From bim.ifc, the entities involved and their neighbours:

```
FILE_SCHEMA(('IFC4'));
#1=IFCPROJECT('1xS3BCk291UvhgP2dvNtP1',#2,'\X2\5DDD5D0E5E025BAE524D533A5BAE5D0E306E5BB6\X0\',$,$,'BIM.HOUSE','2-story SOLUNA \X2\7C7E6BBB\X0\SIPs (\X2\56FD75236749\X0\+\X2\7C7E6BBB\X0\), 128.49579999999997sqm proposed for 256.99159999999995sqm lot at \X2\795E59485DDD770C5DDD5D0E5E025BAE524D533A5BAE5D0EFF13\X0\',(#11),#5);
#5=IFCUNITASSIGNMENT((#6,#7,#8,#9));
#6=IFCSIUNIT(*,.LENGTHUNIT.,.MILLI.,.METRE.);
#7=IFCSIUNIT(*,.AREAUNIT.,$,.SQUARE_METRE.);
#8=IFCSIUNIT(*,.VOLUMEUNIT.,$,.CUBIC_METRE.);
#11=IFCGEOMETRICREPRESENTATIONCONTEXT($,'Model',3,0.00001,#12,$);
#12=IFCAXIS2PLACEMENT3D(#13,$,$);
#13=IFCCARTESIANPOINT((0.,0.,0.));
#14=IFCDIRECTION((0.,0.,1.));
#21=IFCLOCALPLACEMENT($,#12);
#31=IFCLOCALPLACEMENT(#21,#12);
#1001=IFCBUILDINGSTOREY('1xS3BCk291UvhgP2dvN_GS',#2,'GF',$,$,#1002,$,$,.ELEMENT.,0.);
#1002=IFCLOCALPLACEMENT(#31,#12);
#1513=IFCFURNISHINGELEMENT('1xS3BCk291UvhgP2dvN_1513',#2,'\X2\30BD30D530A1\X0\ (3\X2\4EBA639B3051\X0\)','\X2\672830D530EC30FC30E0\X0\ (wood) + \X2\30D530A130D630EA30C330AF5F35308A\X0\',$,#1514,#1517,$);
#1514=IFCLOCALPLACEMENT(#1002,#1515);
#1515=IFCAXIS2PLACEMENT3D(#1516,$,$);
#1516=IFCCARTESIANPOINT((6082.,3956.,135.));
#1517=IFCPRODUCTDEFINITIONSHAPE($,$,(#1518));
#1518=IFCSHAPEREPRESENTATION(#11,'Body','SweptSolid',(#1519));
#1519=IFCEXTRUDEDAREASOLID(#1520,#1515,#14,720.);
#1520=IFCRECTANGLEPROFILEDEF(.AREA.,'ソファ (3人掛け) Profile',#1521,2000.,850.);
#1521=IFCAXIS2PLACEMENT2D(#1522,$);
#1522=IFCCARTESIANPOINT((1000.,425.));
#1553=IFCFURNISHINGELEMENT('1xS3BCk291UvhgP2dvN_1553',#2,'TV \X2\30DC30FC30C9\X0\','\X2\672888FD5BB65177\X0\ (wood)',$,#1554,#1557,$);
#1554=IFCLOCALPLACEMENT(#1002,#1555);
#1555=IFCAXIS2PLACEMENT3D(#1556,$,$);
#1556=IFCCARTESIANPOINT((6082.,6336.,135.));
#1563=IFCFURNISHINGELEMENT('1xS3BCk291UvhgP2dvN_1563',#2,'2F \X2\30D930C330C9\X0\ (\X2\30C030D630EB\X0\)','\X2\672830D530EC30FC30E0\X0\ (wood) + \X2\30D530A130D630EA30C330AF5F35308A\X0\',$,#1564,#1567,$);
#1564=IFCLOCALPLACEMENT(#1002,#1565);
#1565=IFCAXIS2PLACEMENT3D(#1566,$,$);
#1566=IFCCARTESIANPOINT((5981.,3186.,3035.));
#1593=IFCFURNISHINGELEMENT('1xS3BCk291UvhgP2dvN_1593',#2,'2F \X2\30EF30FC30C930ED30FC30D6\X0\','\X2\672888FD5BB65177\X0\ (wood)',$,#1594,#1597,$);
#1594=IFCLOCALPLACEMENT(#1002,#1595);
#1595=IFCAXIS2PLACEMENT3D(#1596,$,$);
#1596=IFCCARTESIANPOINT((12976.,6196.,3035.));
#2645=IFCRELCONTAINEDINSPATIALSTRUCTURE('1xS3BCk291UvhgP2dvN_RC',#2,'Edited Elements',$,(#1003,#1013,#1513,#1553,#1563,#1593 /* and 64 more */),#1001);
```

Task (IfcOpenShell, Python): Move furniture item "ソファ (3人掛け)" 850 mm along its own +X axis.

```python
import ifcopenshell
import ifcopenshell.api.geometry
import ifcopenshell.util.placement
import ifcopenshell.util.unit

model = ifcopenshell.open("bim.ifc")
unit_scale = ifcopenshell.util.unit.calculate_unit_scale(model)

item = model.by_guid("1xS3BCk291UvhgP2dvN_1513")
matrix = ifcopenshell.util.placement.get_local_placement(item.ObjectPlacement)
matrix[:3, 3] += matrix[:3, 0] * 0.85 / unit_scale
ifcopenshell.api.geometry.edit_object_placement(model, product=item, matrix=matrix, is_si=False)

print(ifcopenshell.util.placement.get_local_placement(item.ObjectPlacement).round(3) + 0.0)

model.write("bim_edited.ifc")
```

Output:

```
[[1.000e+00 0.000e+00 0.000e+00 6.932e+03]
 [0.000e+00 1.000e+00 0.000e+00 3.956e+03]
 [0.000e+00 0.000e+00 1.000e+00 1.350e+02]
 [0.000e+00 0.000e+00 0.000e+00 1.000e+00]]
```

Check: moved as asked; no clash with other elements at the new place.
